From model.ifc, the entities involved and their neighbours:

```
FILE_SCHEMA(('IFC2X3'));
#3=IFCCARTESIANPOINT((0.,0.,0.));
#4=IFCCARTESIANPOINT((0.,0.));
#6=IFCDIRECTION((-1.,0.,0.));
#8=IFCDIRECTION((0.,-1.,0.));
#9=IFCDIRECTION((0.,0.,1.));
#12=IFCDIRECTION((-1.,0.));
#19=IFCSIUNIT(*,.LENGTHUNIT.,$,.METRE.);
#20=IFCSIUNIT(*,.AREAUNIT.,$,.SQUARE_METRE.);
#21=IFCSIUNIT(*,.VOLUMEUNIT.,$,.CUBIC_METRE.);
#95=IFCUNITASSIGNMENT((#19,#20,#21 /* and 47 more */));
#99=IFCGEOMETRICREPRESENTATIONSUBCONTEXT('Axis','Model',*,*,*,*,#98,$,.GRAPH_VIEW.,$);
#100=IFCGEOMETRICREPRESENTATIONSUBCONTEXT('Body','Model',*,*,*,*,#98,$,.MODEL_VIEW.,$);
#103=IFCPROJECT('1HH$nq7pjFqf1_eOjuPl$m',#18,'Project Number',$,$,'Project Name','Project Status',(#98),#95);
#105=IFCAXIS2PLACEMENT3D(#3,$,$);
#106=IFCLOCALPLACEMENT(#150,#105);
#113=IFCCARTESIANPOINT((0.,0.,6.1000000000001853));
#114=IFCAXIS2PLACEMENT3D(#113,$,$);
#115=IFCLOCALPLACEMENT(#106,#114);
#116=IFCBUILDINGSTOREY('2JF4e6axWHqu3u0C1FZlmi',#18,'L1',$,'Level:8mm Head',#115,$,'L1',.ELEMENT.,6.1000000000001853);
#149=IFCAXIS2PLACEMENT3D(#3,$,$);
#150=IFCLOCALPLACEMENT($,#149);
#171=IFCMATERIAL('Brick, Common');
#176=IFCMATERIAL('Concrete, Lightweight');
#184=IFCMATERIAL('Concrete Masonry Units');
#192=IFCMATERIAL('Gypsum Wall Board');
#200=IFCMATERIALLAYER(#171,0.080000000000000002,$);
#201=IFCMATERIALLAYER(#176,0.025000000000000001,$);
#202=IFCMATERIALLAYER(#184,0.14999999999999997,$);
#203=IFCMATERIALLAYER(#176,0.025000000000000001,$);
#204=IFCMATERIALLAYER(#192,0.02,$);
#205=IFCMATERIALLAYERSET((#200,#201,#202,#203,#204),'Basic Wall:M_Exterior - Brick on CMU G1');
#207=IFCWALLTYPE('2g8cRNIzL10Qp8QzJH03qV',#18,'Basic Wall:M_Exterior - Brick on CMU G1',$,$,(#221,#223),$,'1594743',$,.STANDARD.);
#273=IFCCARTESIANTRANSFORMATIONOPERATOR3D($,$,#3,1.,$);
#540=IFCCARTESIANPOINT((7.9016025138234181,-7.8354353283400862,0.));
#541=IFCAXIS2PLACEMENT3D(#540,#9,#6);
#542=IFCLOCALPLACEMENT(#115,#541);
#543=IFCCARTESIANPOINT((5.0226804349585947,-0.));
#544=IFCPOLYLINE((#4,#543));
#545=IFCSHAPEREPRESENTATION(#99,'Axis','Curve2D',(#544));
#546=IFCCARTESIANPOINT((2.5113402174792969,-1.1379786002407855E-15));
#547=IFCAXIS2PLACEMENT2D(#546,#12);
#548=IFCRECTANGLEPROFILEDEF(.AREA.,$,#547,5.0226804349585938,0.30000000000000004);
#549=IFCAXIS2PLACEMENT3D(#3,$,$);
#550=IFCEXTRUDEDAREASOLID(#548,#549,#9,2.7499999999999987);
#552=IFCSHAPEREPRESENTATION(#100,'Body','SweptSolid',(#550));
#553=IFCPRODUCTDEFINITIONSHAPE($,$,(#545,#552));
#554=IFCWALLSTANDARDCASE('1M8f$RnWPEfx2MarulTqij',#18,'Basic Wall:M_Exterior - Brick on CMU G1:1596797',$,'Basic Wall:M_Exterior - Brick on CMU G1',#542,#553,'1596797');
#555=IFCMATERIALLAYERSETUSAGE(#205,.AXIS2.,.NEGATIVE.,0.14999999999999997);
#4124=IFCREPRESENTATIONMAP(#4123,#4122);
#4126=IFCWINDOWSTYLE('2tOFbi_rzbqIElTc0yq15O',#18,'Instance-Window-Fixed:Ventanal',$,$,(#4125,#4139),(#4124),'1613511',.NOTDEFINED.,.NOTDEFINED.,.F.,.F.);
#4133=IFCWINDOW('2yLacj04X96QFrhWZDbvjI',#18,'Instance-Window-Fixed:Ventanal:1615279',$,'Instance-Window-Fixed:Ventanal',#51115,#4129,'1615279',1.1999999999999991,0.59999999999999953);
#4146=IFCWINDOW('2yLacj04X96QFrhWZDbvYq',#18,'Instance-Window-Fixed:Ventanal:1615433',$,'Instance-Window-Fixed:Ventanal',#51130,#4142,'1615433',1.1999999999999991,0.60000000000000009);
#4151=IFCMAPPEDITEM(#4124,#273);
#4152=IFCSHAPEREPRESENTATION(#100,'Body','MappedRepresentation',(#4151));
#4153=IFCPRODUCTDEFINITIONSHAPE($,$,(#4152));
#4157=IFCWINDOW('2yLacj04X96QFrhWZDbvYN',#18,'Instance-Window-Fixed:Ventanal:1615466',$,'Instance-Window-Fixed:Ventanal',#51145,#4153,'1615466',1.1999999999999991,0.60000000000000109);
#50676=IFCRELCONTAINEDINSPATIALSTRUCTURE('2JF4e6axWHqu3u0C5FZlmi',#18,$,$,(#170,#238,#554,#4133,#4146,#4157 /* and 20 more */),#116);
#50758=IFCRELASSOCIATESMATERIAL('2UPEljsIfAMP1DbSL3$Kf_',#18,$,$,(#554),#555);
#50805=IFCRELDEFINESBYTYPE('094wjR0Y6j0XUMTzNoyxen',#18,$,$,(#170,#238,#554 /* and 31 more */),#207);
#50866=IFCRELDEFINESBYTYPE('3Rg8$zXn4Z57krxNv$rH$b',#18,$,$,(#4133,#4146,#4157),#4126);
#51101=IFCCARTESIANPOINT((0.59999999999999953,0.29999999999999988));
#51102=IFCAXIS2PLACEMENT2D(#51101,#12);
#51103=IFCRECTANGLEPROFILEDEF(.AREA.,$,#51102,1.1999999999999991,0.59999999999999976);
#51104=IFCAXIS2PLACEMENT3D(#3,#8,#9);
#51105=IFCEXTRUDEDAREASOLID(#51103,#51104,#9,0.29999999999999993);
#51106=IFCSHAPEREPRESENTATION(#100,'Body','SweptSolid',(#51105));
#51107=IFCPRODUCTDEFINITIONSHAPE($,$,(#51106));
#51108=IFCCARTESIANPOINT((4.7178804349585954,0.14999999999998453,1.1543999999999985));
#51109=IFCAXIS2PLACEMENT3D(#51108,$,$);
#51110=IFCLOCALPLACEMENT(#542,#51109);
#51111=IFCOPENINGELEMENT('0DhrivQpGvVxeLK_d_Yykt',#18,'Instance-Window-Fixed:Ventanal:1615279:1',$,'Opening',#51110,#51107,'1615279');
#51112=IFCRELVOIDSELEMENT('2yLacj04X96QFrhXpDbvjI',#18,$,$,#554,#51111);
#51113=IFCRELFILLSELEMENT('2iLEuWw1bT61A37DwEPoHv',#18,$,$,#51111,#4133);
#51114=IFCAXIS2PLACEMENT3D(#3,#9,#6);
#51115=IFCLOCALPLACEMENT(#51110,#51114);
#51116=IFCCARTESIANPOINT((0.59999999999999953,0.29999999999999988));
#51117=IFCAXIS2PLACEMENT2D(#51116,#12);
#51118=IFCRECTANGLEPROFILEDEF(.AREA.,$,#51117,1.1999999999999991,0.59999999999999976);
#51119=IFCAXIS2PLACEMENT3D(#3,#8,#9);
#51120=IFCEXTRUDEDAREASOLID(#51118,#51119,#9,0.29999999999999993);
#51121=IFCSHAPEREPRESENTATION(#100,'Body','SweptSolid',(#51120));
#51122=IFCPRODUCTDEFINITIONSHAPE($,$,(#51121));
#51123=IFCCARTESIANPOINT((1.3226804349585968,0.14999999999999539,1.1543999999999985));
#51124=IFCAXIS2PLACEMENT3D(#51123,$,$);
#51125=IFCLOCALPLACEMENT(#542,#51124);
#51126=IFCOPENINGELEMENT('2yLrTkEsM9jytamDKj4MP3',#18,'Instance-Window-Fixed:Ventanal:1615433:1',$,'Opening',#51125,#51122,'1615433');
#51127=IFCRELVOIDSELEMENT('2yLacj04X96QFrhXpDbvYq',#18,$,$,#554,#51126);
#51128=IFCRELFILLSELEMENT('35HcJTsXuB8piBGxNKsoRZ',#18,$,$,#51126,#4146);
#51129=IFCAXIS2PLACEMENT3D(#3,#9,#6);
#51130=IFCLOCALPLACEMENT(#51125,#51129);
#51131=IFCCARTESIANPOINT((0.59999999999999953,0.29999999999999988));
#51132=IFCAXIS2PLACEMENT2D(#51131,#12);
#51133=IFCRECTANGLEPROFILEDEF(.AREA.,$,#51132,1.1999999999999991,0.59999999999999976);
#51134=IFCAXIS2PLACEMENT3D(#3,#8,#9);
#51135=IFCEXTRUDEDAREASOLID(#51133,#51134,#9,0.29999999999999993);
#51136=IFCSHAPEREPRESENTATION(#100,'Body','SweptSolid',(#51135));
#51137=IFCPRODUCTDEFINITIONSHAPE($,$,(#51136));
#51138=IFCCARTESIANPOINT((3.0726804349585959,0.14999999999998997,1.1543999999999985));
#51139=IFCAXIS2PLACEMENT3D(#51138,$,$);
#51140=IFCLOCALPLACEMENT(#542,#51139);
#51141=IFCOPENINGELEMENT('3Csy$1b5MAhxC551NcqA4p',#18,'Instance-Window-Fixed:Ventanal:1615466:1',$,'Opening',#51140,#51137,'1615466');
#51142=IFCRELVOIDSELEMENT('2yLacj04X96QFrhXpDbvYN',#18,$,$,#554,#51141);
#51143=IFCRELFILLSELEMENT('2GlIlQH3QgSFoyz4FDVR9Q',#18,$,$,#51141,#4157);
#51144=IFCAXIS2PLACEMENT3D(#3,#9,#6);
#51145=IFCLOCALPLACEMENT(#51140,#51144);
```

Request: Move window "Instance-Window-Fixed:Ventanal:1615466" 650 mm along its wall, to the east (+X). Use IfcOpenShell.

```python
import ifcopenshell
import ifcopenshell.api.geometry
import ifcopenshell.util.placement
import ifcopenshell.util.unit

model = ifcopenshell.open("model.ifc")
unit_scale = ifcopenshell.util.unit.calculate_unit_scale(model)

window = model.by_guid("2yLacj04X96QFrhWZDbvYN")
opening = window.FillsVoids[0].RelatingOpeningElement
wall = opening.VoidsElements[0].RelatingBuildingElement

wall_matrix = ifcopenshell.util.placement.get_local_placement(wall.ObjectPlacement)
shift = wall_matrix[:3, 0] * -0.65 / unit_scale
before = ifcopenshell.util.placement.get_local_placement(window.ObjectPlacement)[:3, 3].copy()

# The window is placed relative to its opening, so it follows when the opening moves.
matrix = ifcopenshell.util.placement.get_local_placement(opening.ObjectPlacement)
matrix[:3, 3] += shift
ifcopenshell.api.geometry.edit_object_placement(
    model, product=opening, matrix=matrix, is_si=False, should_transform_children=True
)

after = ifcopenshell.util.placement.get_local_placement(window.ObjectPlacement)[:3, 3]
print("window moved by", (after - before).round(3) + 0.0)

model.write("model_edited.ifc")
```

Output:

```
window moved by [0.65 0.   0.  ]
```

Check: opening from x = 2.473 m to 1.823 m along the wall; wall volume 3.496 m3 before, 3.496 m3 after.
